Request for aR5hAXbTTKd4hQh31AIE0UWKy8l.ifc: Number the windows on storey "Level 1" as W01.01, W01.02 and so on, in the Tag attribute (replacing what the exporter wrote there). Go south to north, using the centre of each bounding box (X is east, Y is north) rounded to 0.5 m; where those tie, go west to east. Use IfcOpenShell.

First a look at what the model holds.

```python
import ifcopenshell
import ifcopenshell.util.element
import ifcopenshell.util.placement

model = ifcopenshell.open("aR5hAXbTTKd4hQh31AIE0UWKy8l.ifc")
print(model.schema)
storey = next(s for s in model.by_type("IfcBuildingStorey") if s.Name == "Level 1")
windows = [e for e in ifcopenshell.util.element.get_decomposition(storey) if e.is_a("IfcWindow")]
for e in sorted(windows, key=lambda e: e.id()):
    origin = ifcopenshell.util.placement.get_local_placement(e.ObjectPlacement)[:3, 3]
    print(e.id(), e.Tag, e.Name, origin.round(2) + 0.0, sep=" | ")
```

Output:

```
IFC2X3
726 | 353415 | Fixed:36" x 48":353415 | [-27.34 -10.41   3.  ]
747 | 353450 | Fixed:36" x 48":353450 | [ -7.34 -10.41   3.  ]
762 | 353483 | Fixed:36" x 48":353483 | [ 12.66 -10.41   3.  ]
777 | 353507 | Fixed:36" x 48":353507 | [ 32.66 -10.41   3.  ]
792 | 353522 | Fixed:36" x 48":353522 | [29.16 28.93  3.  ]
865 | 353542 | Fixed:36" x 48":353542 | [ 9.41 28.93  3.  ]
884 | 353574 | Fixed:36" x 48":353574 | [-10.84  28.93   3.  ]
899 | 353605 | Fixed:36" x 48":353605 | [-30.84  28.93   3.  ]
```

```python
import ifcopenshell
import ifcopenshell.geom
import ifcopenshell.util.element
import ifcopenshell.util.shape

model = ifcopenshell.open("aR5hAXbTTKd4hQh31AIE0UWKy8l.ifc")
settings = ifcopenshell.geom.settings()
settings.set("use-world-coords", True)


def centre(element):
    shape = ifcopenshell.geom.create_shape(settings, element)
    return ifcopenshell.util.shape.get_bbox_centroid(shape.geometry)


storey = next(s for s in model.by_type("IfcBuildingStorey") if s.Name == "Level 1")
windows = [e for e in ifcopenshell.util.element.get_decomposition(storey) if e.is_a("IfcWindow")]

# Insertion points can sit at a corner or the storey origin, so sort by the geometry (in metres).
centres = {e: centre(e) for e in windows}
windows.sort(key=lambda e: (round(centres[e][1] / 0.5), centres[e][0]))

for i, e in enumerate(windows, start=1):
    number = f"W01.{i:02d}"
    e.Tag = number
    print(e.id(), number)

model.write("aR5hAXbTTKd4hQh31AIE0UWKy8l_updated.ifc")
```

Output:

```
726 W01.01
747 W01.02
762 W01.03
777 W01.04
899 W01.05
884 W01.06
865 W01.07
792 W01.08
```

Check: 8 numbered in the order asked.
